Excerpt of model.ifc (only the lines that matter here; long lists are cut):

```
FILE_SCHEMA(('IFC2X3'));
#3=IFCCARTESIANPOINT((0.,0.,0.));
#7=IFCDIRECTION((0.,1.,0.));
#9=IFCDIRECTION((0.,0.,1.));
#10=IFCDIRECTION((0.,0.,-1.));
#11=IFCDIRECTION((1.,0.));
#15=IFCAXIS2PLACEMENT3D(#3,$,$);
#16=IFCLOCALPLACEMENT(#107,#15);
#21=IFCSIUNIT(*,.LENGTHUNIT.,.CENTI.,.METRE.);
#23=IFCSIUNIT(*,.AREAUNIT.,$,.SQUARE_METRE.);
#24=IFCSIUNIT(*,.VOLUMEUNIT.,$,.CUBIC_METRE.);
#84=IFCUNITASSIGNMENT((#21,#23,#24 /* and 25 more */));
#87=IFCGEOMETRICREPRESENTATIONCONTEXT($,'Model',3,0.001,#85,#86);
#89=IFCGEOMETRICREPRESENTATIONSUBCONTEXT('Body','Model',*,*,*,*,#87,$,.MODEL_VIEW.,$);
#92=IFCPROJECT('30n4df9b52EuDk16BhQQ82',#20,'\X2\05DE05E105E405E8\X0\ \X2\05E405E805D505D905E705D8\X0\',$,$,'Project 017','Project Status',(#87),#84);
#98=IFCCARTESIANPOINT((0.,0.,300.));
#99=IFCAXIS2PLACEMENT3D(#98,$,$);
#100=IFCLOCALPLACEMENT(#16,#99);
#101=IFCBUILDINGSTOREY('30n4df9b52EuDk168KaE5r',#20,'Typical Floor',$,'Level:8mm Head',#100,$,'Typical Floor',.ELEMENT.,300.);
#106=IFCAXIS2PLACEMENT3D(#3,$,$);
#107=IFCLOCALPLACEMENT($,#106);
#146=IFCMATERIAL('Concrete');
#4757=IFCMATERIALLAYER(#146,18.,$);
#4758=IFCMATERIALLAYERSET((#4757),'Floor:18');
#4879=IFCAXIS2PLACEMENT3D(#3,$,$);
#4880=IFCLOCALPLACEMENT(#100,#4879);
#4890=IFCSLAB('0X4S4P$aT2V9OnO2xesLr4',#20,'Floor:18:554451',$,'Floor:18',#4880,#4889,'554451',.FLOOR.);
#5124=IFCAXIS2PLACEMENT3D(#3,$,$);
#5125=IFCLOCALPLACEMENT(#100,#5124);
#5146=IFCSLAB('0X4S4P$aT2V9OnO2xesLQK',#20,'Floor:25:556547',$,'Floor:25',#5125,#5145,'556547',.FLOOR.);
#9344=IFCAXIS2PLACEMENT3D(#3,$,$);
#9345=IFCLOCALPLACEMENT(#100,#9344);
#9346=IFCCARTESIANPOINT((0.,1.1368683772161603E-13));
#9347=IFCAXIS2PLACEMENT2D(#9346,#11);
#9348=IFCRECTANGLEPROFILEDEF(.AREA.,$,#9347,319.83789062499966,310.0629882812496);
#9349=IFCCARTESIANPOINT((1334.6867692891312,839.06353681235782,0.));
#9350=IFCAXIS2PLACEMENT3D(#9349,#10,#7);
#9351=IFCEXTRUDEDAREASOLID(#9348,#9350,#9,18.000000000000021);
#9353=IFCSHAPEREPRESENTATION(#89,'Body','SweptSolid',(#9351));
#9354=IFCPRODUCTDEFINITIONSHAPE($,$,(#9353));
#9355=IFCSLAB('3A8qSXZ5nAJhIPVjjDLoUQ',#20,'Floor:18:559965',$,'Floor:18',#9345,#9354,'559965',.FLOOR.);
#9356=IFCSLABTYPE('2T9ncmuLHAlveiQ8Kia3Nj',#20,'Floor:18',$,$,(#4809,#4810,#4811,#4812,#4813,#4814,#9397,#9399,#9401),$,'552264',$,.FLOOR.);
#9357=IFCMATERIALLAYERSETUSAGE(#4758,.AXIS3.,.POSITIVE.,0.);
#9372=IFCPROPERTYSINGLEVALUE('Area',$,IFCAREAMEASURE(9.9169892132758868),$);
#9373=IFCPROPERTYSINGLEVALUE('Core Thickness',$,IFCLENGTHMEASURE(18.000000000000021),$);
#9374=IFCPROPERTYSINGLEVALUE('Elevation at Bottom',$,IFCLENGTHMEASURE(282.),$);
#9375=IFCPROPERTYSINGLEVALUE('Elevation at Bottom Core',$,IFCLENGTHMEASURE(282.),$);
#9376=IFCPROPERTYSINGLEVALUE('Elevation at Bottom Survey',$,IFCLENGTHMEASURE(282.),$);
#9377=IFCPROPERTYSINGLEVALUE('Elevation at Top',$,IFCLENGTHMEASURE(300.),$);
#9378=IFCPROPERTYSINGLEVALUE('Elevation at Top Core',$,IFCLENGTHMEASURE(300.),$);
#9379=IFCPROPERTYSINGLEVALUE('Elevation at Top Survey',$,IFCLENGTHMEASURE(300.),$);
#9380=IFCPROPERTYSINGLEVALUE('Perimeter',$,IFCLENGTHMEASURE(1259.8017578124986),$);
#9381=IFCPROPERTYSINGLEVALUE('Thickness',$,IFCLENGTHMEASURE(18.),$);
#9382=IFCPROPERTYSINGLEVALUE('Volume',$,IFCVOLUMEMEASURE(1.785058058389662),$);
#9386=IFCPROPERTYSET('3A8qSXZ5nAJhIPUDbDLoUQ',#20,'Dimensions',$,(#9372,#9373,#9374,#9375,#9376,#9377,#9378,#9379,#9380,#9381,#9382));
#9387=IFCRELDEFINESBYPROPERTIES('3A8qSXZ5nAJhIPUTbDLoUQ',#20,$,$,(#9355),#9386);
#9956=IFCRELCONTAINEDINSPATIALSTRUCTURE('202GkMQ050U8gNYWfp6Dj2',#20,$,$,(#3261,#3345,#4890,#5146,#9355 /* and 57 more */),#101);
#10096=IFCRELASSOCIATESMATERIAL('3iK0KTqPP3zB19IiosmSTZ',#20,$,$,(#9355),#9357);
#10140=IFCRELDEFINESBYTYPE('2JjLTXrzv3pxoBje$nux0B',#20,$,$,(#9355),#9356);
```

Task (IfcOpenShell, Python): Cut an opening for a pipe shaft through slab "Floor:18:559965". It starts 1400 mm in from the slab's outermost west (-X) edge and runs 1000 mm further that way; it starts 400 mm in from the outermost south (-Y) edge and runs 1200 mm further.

```python
import numpy as np
import ifcopenshell
import ifcopenshell.api.feature
import ifcopenshell.api.geometry
import ifcopenshell.api.pset
import ifcopenshell.api.root
import ifcopenshell.geom
import ifcopenshell.util.element
import ifcopenshell.util.placement
import ifcopenshell.util.representation
import ifcopenshell.util.shape
import ifcopenshell.util.unit

model = ifcopenshell.open("model.ifc")
unit_scale = ifcopenshell.util.unit.calculate_unit_scale(model)
area_scale = ifcopenshell.util.unit.calculate_unit_scale(model, "AREAUNIT")
volume_scale = ifcopenshell.util.unit.calculate_unit_scale(model, "VOLUMEUNIT")
settings = ifcopenshell.geom.settings()


def volume(element):
    """Net volume in cubic metres, openings subtracted."""
    shape = ifcopenshell.geom.create_shape(settings, element)
    return ifcopenshell.util.shape.get_volume(shape.geometry)


slab = model.by_id(9355)
before = volume(slab)

# Extent in the slab's own axes, in metres. The edges named are its -X and -Y sides.
slab_shape = ifcopenshell.geom.create_shape(settings, slab)
vertices = ifcopenshell.util.shape.get_vertices(slab_shape.geometry)
x_min, y_min, bottom = vertices.min(axis=0)
top = vertices[:, 2].max()

opening = ifcopenshell.api.root.create_entity(model, ifc_class="IfcOpeningElement", name="Pipe shaft opening")
context = ifcopenshell.util.representation.get_context(model, "Model", "Body", "MODEL_VIEW")
width, depth = 1, 1.2
outline = [(0.0, 0.0), (width, 0.0), (width, depth), (0.0, depth), (0.0, 0.0)]
# Overshoot both faces by 50 mm so the cut is clean.
shape = ifcopenshell.api.geometry.add_slab_representation(
    model, context=context, depth=top - bottom + 0.1, polyline=outline
)
ifcopenshell.api.geometry.assign_representation(model, product=opening, representation=shape)

matrix = ifcopenshell.util.placement.get_local_placement(slab.ObjectPlacement)
matrix[:, 3] = matrix @ np.append(np.array([x_min + 1.4, y_min + 0.4, bottom - 0.05]) / unit_scale, 1.0)
ifcopenshell.api.geometry.edit_object_placement(model, product=opening, matrix=matrix, is_si=False)
ifcopenshell.api.feature.add_feature(model, feature=opening, element=slab)

after = volume(slab)

# Update the slab's stored quantities.
pset = model.by_id(ifcopenshell.util.element.get_pset(slab, "Dimensions", should_inherit=False)["id"])
ifcopenshell.api.pset.edit_pset(model, pset=pset, properties={
    "Area": model.create_entity("IfcAreaMeasure", after / (top - bottom) / area_scale),
    "Volume": model.create_entity("IfcVolumeMeasure", after / volume_scale),
})

print(f"slab volume {before:.3f} -> {after:.3f} m3")

model.write("model-out.ifc")
```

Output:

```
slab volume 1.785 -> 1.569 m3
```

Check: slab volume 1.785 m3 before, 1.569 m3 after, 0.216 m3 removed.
